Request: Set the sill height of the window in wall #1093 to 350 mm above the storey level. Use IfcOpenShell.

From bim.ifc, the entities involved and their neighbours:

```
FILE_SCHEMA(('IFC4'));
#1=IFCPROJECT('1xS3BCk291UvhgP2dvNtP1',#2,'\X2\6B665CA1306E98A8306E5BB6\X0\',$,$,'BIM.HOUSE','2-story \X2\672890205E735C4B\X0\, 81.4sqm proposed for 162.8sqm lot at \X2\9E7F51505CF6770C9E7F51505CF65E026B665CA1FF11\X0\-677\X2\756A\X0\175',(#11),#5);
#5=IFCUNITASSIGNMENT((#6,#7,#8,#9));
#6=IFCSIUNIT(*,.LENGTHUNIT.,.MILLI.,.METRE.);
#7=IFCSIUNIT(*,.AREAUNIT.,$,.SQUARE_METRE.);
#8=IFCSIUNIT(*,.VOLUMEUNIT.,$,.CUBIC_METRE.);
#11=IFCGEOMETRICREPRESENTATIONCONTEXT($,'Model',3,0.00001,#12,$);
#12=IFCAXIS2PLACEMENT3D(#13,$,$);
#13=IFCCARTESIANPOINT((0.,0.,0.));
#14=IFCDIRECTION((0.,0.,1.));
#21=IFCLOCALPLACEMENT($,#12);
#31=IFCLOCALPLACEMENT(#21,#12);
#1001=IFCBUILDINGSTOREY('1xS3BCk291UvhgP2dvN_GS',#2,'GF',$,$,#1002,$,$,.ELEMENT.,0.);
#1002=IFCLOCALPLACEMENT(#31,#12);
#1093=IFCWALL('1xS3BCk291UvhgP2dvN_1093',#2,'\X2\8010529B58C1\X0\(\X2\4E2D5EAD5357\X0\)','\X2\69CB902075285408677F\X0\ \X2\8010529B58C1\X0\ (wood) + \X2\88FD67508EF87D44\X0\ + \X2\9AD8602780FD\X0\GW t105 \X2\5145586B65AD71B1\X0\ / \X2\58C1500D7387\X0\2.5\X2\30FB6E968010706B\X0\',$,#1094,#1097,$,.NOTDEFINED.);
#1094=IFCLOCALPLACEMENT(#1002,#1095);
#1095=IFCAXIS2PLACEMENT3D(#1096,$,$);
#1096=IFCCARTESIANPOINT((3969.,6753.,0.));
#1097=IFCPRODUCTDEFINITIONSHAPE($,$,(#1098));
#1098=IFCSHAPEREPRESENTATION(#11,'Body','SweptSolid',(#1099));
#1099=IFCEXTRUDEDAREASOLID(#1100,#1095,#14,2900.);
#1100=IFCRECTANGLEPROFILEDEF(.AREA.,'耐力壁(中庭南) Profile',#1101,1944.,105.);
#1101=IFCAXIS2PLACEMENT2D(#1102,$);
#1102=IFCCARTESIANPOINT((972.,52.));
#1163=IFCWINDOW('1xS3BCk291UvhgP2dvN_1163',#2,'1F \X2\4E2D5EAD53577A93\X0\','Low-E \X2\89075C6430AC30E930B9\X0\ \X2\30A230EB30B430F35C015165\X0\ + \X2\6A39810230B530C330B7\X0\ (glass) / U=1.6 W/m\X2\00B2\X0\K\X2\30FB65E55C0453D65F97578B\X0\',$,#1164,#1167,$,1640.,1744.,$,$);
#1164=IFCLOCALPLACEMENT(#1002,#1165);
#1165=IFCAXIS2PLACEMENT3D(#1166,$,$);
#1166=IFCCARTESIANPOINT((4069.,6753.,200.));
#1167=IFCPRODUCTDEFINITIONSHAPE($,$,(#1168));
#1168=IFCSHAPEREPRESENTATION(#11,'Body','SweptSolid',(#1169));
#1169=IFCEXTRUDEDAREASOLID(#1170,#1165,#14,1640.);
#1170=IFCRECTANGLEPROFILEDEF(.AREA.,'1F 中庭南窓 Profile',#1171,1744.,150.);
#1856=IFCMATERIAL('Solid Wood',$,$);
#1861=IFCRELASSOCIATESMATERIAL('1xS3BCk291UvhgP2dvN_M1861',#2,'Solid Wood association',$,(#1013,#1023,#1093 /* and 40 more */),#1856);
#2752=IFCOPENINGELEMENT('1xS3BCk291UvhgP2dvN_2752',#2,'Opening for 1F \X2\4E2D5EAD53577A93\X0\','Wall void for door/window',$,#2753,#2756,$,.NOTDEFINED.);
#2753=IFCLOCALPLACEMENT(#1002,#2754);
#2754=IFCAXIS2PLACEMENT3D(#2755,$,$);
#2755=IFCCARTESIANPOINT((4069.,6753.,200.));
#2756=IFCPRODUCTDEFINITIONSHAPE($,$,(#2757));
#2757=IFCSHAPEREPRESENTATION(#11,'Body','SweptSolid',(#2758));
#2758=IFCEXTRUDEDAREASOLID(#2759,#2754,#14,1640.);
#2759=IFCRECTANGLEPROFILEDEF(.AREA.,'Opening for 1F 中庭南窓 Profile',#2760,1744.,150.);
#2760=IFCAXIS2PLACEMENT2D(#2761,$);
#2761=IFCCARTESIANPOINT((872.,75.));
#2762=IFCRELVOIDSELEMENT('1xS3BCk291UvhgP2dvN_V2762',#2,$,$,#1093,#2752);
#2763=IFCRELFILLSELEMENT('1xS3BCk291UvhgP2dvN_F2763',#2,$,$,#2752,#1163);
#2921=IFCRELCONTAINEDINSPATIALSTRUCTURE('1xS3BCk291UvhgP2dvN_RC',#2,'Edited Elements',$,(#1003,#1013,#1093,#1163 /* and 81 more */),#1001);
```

```python
import numpy as np
import ifcopenshell
import ifcopenshell.api.geometry
import ifcopenshell.geom
import ifcopenshell.util.element
import ifcopenshell.util.placement
import ifcopenshell.util.shape
import ifcopenshell.util.unit

model = ifcopenshell.open("bim.ifc")
unit_scale = ifcopenshell.util.unit.calculate_unit_scale(model)

window = model.by_id(1163)
opening = window.FillsVoids[0].RelatingOpeningElement
storey = ifcopenshell.util.element.get_container(window, ifc_class="IfcBuildingStorey")
level = ifcopenshell.util.placement.get_local_placement(storey.ObjectPlacement)[2, 3]

# The opening's origin need not be at the sill, so measure its lowest point.
shape = ifcopenshell.geom.create_shape(ifcopenshell.geom.settings(), opening)
bottom = ifcopenshell.util.shape.get_shape_bottom_elevation(shape, shape.geometry) / unit_scale
dz = level + 0.35 / unit_scale - bottom

shift = np.array([0.0, 0.0, dz])
# The window is not placed relative to its opening, so move both.
for product in (opening, window):
    matrix = ifcopenshell.util.placement.get_local_placement(product.ObjectPlacement)
    matrix[:3, 3] += shift
    ifcopenshell.api.geometry.edit_object_placement(model, product=product, matrix=matrix, is_si=False)

print(f"moved by {dz * unit_scale:+.3f} m")

model.write("bim_rev.ifc")
```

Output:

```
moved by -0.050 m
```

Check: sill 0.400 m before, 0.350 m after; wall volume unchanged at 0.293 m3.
